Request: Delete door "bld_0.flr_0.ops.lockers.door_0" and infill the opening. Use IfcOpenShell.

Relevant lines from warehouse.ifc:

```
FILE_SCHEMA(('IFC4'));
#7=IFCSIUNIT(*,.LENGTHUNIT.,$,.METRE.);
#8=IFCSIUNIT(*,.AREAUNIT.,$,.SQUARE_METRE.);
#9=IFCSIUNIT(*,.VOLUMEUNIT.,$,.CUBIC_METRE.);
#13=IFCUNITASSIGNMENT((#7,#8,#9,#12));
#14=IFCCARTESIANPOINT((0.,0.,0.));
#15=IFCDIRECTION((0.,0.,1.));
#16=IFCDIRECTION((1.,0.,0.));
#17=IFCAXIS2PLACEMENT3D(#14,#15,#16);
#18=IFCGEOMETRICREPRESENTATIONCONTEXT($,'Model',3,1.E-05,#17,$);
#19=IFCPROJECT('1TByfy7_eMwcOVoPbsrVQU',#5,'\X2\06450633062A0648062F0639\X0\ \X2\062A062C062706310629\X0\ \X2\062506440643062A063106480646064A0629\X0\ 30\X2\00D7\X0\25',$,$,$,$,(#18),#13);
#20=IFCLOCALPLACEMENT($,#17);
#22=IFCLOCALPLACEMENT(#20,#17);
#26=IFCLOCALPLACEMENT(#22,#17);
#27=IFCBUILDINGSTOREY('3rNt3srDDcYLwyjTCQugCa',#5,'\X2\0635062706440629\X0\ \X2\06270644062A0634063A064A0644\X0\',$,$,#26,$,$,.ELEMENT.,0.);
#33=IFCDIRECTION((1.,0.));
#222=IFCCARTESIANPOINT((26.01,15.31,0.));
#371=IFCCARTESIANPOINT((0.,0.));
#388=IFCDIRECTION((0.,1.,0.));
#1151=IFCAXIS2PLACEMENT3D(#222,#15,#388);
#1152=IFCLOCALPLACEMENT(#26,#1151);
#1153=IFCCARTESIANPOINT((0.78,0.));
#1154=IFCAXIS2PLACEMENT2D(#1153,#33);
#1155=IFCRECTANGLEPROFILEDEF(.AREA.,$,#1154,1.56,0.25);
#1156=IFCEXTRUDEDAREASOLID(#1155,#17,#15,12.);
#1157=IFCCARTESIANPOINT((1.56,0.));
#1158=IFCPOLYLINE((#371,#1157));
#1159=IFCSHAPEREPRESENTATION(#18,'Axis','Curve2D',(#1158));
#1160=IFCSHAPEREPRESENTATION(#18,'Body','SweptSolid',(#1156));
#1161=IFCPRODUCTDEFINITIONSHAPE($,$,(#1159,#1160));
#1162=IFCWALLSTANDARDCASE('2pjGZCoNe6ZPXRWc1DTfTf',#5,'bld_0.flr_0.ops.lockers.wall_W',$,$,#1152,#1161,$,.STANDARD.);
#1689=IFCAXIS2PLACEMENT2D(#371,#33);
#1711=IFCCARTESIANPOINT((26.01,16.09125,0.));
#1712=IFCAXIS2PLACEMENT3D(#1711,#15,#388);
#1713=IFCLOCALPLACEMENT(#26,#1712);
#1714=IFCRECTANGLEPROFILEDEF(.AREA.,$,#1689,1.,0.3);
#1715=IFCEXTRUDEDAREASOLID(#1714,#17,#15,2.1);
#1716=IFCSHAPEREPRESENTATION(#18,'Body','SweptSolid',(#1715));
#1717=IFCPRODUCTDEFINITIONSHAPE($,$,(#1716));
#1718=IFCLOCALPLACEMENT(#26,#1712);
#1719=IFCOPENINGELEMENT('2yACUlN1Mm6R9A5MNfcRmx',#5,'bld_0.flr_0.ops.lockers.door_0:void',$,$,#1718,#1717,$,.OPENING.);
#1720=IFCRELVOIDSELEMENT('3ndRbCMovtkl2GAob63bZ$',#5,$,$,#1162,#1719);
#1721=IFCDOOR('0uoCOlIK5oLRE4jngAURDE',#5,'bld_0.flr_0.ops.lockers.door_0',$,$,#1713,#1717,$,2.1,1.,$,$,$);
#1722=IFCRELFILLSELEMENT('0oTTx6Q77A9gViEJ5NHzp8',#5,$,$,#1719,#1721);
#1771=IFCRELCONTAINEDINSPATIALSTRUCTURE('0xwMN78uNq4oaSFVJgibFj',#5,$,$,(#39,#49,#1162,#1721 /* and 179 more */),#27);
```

```python
import ifcopenshell
import ifcopenshell.api.feature
import ifcopenshell.api.root
import ifcopenshell.geom
import ifcopenshell.util.shape

model = ifcopenshell.open("warehouse.ifc")
settings = ifcopenshell.geom.settings()


def volume(element):
    """Net volume in cubic metres, openings subtracted."""
    shape = ifcopenshell.geom.create_shape(settings, element)
    return ifcopenshell.util.shape.get_volume(shape.geometry)


door = model.by_guid("0uoCOlIK5oLRE4jngAURDE")
opening = door.FillsVoids[0].RelatingOpeningElement
wall = opening.VoidsElements[0].RelatingBuildingElement
before = volume(wall)

ifcopenshell.api.root.remove_product(model, product=door)
ifcopenshell.api.feature.remove_feature(model, feature=opening)

after = volume(wall)

print(f"wall volume {before:.3f} -> {after:.3f} m3")

model.write("warehouse_rev.ifc")
```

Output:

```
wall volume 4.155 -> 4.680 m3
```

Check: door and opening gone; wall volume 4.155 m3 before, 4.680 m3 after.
